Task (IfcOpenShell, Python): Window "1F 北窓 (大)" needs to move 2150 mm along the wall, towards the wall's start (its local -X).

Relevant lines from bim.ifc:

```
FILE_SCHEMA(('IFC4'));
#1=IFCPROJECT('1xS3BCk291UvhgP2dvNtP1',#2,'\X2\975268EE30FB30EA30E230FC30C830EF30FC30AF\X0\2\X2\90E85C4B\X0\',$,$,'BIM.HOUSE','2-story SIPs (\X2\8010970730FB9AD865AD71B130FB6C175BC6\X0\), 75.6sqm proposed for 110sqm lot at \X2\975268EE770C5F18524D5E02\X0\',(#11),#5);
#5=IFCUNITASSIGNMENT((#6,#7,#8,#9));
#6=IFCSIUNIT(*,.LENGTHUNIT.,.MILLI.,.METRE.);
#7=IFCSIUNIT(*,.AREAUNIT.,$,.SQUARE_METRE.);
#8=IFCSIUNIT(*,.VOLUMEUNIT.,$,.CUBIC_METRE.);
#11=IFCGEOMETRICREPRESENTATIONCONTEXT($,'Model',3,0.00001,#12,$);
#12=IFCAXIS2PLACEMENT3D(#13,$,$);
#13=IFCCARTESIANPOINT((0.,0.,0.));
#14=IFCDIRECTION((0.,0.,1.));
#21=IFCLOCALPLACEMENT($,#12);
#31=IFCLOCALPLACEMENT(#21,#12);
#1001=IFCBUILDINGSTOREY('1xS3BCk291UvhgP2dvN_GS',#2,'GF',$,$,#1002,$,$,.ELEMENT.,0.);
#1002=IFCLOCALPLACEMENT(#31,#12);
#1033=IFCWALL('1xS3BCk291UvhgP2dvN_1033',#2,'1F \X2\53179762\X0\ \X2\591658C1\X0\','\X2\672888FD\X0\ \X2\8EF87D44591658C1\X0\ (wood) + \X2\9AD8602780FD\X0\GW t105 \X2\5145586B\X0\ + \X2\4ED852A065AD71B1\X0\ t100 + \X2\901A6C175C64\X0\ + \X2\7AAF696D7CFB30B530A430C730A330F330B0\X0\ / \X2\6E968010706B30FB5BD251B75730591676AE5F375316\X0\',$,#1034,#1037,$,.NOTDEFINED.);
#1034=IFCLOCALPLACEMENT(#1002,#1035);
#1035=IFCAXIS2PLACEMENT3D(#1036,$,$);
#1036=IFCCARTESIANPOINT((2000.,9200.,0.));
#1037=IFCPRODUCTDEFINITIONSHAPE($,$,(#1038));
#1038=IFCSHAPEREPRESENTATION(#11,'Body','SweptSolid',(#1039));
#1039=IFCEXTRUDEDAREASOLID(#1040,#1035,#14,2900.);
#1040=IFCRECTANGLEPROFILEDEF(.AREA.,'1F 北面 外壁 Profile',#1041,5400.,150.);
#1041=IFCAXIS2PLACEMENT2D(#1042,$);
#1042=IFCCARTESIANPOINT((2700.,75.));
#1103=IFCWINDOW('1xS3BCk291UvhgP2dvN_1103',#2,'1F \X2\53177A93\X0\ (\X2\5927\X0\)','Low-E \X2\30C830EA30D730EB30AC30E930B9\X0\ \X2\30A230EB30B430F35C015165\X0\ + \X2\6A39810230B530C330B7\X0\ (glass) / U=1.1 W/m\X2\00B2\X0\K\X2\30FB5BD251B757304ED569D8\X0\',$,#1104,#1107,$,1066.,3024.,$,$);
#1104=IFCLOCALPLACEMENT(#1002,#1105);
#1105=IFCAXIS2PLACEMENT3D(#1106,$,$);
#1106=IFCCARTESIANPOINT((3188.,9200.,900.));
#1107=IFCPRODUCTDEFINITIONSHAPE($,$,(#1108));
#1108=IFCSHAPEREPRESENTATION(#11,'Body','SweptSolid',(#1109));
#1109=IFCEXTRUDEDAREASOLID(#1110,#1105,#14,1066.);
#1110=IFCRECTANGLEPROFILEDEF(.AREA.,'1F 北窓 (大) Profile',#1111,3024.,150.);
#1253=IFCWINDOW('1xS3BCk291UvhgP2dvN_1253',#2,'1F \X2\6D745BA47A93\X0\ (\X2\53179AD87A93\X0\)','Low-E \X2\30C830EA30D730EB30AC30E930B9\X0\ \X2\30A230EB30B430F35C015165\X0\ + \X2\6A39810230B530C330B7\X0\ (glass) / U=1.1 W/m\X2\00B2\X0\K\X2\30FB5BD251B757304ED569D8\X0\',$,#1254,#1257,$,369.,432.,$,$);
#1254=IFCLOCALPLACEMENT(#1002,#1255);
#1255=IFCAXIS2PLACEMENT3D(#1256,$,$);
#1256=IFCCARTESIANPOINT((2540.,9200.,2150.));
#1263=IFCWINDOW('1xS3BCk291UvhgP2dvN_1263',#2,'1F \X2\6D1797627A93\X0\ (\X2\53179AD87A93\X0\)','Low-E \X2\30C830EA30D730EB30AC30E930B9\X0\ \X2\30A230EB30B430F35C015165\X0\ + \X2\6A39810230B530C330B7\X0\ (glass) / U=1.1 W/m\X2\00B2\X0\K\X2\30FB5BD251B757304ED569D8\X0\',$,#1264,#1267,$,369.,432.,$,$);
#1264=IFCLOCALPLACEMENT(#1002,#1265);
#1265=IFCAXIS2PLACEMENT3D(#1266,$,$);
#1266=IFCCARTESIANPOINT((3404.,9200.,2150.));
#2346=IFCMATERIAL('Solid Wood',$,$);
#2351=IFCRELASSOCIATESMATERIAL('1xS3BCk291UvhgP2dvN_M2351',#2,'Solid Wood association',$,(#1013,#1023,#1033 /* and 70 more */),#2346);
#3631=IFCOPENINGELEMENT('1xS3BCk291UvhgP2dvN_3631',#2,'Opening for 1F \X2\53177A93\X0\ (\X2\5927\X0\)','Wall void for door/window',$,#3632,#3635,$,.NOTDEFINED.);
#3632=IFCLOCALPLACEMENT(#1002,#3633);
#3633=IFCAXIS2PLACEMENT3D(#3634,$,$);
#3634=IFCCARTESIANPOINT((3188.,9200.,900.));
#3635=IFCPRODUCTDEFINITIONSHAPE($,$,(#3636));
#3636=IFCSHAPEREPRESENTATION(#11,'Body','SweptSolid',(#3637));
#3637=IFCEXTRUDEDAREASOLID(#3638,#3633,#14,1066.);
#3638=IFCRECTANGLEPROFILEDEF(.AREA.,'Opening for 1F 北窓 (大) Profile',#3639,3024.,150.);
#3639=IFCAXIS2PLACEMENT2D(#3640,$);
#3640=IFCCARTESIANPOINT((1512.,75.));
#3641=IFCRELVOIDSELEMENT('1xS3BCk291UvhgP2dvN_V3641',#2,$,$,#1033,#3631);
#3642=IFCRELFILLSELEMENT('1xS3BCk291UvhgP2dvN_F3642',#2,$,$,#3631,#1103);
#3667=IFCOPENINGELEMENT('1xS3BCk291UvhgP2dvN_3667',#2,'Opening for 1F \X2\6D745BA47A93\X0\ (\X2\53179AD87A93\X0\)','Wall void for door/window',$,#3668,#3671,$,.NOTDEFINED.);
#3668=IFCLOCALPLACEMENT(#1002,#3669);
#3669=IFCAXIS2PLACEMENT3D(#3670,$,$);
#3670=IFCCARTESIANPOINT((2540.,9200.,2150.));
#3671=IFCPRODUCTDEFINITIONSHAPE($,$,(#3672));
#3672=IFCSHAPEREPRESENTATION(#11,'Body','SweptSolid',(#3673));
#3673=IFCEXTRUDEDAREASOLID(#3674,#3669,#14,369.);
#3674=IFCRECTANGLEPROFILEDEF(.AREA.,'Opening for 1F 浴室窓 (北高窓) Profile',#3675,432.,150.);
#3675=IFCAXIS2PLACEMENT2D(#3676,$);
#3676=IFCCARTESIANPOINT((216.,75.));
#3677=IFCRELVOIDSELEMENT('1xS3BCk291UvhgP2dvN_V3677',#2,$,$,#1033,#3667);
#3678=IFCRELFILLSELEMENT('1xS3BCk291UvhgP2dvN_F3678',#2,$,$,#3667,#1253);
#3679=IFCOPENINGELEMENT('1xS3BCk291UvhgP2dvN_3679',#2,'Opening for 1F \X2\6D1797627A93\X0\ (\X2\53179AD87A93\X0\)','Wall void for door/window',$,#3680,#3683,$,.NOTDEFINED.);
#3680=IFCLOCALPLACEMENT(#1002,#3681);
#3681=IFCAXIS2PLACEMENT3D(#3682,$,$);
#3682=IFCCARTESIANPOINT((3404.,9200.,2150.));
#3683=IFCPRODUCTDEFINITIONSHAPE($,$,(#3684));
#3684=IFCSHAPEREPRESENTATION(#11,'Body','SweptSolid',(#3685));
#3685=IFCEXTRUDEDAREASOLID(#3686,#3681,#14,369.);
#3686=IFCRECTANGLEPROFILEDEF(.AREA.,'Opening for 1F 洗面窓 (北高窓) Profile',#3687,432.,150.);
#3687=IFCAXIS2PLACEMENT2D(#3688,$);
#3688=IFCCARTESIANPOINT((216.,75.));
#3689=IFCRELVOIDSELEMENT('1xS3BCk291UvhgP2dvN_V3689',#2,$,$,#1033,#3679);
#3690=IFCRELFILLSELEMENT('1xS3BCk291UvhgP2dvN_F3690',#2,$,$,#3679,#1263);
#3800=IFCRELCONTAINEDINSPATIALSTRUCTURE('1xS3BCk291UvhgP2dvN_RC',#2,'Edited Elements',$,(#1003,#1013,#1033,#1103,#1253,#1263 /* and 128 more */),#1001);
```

```python
import ifcopenshell
import ifcopenshell.api.geometry
import ifcopenshell.util.placement
import ifcopenshell.util.unit

model = ifcopenshell.open("bim.ifc")
unit_scale = ifcopenshell.util.unit.calculate_unit_scale(model)

window = model.by_guid("1xS3BCk291UvhgP2dvN_1103")
opening = window.FillsVoids[0].RelatingOpeningElement
wall = opening.VoidsElements[0].RelatingBuildingElement

wall_matrix = ifcopenshell.util.placement.get_local_placement(wall.ObjectPlacement)
shift = wall_matrix[:3, 0] * -2.15 / unit_scale
before = ifcopenshell.util.placement.get_local_placement(window.ObjectPlacement)[:3, 3].copy()

# The window is not placed relative to its opening, so move both.
for product in (opening, window):
    matrix = ifcopenshell.util.placement.get_local_placement(product.ObjectPlacement)
    matrix[:3, 3] += shift
    ifcopenshell.api.geometry.edit_object_placement(model, product=product, matrix=matrix, is_si=False)

after = ifcopenshell.util.placement.get_local_placement(window.ObjectPlacement)[:3, 3]
print("window moved by", (after - before).round(3) + 0.0)

model.write("bim_v2.ifc")
```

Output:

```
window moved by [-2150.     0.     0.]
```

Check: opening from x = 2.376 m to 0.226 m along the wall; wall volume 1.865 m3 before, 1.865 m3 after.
